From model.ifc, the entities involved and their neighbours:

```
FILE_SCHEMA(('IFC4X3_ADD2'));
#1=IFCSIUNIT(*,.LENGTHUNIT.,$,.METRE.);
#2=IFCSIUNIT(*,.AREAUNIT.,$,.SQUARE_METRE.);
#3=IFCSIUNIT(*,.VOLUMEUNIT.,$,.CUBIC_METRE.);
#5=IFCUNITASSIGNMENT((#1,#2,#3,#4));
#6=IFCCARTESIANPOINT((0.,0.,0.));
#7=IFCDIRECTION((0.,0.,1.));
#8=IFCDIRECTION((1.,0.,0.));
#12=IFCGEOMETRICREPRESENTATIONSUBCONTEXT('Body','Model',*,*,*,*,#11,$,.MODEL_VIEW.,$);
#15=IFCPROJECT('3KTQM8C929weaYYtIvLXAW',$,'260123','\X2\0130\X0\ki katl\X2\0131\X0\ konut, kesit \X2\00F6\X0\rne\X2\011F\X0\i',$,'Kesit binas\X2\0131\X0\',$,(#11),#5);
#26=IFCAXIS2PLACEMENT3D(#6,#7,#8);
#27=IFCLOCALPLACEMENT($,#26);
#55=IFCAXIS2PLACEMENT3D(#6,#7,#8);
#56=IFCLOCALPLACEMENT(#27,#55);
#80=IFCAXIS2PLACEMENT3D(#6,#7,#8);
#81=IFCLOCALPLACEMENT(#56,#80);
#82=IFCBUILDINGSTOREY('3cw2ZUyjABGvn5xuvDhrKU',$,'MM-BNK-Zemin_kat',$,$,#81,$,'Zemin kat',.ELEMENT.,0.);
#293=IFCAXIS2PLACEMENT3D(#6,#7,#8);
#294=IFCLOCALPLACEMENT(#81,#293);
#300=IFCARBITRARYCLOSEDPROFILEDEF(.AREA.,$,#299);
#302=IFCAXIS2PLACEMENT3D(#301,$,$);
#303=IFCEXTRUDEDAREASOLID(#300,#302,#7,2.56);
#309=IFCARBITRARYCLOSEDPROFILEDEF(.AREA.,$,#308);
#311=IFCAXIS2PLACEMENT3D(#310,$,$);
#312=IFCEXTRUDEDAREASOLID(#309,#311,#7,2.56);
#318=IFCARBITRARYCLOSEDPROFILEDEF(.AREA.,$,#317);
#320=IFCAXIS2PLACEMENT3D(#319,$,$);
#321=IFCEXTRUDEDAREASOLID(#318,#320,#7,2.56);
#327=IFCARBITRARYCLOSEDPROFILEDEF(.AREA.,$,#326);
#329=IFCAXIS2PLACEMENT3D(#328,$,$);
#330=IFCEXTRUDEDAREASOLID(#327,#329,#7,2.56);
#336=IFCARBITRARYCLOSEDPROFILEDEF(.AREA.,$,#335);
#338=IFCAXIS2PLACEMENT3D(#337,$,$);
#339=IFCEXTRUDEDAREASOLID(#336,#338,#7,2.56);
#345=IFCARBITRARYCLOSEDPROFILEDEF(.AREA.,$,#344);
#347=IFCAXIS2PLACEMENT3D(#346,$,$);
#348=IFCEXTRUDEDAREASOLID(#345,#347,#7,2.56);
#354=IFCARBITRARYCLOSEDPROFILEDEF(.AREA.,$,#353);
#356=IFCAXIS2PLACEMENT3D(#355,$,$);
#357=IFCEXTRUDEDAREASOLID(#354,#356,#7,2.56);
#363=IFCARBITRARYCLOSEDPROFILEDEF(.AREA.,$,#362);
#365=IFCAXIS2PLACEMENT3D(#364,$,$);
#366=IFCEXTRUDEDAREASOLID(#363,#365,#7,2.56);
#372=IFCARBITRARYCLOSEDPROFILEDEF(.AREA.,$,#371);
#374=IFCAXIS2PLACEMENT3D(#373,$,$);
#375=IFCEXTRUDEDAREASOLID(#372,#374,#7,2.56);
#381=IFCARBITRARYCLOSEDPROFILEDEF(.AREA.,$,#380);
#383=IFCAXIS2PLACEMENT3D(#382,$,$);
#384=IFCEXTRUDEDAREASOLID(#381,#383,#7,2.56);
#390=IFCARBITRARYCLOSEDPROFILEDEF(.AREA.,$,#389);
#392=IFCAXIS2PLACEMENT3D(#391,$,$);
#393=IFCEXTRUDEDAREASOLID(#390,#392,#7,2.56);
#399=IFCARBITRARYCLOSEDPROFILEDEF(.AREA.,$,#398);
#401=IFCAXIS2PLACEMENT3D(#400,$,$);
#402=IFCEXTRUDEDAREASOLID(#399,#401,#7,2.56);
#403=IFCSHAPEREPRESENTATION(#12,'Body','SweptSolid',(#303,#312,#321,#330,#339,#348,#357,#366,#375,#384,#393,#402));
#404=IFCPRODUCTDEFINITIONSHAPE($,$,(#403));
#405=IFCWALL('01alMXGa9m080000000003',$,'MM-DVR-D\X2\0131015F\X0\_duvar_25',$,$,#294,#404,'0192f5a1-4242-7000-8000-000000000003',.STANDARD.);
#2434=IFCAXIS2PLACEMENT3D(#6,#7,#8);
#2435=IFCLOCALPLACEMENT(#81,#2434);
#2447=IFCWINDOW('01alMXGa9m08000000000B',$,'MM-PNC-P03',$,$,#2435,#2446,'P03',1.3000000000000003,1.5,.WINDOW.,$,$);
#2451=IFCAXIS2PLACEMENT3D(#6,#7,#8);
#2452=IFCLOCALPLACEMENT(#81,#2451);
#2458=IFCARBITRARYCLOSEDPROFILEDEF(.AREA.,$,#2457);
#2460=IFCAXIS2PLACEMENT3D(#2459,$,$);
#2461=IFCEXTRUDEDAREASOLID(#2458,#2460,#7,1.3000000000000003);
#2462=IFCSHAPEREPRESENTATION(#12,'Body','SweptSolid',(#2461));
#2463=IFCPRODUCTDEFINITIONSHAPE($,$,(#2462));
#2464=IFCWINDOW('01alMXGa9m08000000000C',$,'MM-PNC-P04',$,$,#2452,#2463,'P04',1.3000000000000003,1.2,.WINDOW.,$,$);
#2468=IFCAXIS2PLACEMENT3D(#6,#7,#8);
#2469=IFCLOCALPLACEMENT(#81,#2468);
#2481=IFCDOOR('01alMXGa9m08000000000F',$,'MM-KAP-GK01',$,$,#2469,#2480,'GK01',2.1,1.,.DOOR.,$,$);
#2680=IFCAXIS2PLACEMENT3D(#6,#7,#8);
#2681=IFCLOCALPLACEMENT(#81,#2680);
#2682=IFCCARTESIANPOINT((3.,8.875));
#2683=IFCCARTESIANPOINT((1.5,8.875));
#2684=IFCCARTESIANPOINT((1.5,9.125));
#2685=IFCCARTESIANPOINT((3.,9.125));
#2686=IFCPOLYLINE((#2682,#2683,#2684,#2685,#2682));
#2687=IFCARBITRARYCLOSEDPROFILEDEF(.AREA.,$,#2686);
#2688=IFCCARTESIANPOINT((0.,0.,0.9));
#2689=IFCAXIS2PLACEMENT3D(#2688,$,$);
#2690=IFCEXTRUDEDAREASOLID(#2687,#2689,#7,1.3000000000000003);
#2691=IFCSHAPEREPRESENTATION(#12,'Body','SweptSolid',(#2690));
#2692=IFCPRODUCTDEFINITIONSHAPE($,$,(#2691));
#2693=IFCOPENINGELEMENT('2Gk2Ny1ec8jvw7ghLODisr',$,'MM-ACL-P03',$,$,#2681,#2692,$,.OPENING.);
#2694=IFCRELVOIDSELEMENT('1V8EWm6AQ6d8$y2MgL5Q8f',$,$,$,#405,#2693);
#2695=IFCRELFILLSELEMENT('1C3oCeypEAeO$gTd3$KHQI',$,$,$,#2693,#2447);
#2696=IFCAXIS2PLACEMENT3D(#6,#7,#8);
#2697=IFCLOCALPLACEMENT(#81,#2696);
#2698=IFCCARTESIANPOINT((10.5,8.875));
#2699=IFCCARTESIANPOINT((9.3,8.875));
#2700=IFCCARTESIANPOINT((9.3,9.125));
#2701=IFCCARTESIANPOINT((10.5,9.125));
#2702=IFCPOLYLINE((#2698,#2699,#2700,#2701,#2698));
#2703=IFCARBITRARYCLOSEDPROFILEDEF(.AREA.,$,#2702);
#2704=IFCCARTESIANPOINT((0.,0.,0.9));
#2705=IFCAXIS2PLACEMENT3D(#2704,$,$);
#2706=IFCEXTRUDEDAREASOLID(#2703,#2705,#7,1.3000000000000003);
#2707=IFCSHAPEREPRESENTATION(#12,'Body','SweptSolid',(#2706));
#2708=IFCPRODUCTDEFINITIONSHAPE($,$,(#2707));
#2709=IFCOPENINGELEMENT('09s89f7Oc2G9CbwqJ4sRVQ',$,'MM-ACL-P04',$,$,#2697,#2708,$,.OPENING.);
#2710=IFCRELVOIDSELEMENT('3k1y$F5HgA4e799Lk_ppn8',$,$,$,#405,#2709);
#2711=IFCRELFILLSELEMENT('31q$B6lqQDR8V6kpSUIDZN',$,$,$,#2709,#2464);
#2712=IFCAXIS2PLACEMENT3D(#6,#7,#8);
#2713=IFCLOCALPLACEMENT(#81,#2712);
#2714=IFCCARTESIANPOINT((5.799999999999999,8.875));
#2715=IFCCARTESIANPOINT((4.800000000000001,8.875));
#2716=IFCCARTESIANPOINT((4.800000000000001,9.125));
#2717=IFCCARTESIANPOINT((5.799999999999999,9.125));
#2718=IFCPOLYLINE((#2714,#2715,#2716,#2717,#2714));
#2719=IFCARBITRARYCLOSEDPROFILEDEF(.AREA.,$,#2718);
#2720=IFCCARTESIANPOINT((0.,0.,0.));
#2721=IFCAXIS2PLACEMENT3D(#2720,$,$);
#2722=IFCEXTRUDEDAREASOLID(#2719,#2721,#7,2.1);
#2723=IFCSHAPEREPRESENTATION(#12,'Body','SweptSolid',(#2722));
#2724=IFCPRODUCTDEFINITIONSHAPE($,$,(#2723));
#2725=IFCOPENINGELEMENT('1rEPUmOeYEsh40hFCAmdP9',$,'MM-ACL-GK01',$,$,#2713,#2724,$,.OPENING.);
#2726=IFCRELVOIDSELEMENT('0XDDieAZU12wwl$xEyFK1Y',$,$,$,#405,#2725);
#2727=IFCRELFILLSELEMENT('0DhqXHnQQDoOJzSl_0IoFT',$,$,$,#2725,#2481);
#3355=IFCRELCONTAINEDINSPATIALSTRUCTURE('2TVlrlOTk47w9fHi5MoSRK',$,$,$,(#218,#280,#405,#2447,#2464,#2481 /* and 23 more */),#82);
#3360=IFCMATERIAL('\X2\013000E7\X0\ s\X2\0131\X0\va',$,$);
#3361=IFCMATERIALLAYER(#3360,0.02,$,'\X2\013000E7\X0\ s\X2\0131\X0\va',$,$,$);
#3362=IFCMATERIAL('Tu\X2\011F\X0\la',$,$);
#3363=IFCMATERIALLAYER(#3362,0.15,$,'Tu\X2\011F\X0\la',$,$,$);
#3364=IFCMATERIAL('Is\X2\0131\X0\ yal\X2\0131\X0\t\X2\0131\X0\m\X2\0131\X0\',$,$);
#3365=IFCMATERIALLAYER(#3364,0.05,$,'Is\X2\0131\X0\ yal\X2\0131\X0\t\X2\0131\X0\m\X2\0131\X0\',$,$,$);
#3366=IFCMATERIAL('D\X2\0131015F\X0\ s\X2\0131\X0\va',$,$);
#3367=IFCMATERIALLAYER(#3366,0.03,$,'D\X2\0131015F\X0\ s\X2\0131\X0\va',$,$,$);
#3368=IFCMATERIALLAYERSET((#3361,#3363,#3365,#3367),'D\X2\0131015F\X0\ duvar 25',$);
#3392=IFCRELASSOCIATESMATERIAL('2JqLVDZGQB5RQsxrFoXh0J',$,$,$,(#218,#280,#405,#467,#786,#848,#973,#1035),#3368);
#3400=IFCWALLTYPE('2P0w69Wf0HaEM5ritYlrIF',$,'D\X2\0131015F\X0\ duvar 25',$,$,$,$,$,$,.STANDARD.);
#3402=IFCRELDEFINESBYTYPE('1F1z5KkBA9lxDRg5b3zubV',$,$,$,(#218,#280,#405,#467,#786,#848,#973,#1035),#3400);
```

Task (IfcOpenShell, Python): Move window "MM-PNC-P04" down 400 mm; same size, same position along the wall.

```python
import numpy as np
import ifcopenshell
import ifcopenshell.api.geometry
import ifcopenshell.util.placement
import ifcopenshell.util.unit

model = ifcopenshell.open("model.ifc")
unit_scale = ifcopenshell.util.unit.calculate_unit_scale(model)

window = model.by_id(2464)
opening = window.FillsVoids[0].RelatingOpeningElement
dz = -0.4 / unit_scale

shift = np.array([0.0, 0.0, dz])
# The window is not placed relative to its opening, so move both.
for product in (opening, window):
    matrix = ifcopenshell.util.placement.get_local_placement(product.ObjectPlacement)
    matrix[:3, 3] += shift
    ifcopenshell.api.geometry.edit_object_placement(model, product=product, matrix=matrix, is_si=False)

print(f"moved by {dz * unit_scale:+.3f} m")

model.write("model_v2.ifc")
```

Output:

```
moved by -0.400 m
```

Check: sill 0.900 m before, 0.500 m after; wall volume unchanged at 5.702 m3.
